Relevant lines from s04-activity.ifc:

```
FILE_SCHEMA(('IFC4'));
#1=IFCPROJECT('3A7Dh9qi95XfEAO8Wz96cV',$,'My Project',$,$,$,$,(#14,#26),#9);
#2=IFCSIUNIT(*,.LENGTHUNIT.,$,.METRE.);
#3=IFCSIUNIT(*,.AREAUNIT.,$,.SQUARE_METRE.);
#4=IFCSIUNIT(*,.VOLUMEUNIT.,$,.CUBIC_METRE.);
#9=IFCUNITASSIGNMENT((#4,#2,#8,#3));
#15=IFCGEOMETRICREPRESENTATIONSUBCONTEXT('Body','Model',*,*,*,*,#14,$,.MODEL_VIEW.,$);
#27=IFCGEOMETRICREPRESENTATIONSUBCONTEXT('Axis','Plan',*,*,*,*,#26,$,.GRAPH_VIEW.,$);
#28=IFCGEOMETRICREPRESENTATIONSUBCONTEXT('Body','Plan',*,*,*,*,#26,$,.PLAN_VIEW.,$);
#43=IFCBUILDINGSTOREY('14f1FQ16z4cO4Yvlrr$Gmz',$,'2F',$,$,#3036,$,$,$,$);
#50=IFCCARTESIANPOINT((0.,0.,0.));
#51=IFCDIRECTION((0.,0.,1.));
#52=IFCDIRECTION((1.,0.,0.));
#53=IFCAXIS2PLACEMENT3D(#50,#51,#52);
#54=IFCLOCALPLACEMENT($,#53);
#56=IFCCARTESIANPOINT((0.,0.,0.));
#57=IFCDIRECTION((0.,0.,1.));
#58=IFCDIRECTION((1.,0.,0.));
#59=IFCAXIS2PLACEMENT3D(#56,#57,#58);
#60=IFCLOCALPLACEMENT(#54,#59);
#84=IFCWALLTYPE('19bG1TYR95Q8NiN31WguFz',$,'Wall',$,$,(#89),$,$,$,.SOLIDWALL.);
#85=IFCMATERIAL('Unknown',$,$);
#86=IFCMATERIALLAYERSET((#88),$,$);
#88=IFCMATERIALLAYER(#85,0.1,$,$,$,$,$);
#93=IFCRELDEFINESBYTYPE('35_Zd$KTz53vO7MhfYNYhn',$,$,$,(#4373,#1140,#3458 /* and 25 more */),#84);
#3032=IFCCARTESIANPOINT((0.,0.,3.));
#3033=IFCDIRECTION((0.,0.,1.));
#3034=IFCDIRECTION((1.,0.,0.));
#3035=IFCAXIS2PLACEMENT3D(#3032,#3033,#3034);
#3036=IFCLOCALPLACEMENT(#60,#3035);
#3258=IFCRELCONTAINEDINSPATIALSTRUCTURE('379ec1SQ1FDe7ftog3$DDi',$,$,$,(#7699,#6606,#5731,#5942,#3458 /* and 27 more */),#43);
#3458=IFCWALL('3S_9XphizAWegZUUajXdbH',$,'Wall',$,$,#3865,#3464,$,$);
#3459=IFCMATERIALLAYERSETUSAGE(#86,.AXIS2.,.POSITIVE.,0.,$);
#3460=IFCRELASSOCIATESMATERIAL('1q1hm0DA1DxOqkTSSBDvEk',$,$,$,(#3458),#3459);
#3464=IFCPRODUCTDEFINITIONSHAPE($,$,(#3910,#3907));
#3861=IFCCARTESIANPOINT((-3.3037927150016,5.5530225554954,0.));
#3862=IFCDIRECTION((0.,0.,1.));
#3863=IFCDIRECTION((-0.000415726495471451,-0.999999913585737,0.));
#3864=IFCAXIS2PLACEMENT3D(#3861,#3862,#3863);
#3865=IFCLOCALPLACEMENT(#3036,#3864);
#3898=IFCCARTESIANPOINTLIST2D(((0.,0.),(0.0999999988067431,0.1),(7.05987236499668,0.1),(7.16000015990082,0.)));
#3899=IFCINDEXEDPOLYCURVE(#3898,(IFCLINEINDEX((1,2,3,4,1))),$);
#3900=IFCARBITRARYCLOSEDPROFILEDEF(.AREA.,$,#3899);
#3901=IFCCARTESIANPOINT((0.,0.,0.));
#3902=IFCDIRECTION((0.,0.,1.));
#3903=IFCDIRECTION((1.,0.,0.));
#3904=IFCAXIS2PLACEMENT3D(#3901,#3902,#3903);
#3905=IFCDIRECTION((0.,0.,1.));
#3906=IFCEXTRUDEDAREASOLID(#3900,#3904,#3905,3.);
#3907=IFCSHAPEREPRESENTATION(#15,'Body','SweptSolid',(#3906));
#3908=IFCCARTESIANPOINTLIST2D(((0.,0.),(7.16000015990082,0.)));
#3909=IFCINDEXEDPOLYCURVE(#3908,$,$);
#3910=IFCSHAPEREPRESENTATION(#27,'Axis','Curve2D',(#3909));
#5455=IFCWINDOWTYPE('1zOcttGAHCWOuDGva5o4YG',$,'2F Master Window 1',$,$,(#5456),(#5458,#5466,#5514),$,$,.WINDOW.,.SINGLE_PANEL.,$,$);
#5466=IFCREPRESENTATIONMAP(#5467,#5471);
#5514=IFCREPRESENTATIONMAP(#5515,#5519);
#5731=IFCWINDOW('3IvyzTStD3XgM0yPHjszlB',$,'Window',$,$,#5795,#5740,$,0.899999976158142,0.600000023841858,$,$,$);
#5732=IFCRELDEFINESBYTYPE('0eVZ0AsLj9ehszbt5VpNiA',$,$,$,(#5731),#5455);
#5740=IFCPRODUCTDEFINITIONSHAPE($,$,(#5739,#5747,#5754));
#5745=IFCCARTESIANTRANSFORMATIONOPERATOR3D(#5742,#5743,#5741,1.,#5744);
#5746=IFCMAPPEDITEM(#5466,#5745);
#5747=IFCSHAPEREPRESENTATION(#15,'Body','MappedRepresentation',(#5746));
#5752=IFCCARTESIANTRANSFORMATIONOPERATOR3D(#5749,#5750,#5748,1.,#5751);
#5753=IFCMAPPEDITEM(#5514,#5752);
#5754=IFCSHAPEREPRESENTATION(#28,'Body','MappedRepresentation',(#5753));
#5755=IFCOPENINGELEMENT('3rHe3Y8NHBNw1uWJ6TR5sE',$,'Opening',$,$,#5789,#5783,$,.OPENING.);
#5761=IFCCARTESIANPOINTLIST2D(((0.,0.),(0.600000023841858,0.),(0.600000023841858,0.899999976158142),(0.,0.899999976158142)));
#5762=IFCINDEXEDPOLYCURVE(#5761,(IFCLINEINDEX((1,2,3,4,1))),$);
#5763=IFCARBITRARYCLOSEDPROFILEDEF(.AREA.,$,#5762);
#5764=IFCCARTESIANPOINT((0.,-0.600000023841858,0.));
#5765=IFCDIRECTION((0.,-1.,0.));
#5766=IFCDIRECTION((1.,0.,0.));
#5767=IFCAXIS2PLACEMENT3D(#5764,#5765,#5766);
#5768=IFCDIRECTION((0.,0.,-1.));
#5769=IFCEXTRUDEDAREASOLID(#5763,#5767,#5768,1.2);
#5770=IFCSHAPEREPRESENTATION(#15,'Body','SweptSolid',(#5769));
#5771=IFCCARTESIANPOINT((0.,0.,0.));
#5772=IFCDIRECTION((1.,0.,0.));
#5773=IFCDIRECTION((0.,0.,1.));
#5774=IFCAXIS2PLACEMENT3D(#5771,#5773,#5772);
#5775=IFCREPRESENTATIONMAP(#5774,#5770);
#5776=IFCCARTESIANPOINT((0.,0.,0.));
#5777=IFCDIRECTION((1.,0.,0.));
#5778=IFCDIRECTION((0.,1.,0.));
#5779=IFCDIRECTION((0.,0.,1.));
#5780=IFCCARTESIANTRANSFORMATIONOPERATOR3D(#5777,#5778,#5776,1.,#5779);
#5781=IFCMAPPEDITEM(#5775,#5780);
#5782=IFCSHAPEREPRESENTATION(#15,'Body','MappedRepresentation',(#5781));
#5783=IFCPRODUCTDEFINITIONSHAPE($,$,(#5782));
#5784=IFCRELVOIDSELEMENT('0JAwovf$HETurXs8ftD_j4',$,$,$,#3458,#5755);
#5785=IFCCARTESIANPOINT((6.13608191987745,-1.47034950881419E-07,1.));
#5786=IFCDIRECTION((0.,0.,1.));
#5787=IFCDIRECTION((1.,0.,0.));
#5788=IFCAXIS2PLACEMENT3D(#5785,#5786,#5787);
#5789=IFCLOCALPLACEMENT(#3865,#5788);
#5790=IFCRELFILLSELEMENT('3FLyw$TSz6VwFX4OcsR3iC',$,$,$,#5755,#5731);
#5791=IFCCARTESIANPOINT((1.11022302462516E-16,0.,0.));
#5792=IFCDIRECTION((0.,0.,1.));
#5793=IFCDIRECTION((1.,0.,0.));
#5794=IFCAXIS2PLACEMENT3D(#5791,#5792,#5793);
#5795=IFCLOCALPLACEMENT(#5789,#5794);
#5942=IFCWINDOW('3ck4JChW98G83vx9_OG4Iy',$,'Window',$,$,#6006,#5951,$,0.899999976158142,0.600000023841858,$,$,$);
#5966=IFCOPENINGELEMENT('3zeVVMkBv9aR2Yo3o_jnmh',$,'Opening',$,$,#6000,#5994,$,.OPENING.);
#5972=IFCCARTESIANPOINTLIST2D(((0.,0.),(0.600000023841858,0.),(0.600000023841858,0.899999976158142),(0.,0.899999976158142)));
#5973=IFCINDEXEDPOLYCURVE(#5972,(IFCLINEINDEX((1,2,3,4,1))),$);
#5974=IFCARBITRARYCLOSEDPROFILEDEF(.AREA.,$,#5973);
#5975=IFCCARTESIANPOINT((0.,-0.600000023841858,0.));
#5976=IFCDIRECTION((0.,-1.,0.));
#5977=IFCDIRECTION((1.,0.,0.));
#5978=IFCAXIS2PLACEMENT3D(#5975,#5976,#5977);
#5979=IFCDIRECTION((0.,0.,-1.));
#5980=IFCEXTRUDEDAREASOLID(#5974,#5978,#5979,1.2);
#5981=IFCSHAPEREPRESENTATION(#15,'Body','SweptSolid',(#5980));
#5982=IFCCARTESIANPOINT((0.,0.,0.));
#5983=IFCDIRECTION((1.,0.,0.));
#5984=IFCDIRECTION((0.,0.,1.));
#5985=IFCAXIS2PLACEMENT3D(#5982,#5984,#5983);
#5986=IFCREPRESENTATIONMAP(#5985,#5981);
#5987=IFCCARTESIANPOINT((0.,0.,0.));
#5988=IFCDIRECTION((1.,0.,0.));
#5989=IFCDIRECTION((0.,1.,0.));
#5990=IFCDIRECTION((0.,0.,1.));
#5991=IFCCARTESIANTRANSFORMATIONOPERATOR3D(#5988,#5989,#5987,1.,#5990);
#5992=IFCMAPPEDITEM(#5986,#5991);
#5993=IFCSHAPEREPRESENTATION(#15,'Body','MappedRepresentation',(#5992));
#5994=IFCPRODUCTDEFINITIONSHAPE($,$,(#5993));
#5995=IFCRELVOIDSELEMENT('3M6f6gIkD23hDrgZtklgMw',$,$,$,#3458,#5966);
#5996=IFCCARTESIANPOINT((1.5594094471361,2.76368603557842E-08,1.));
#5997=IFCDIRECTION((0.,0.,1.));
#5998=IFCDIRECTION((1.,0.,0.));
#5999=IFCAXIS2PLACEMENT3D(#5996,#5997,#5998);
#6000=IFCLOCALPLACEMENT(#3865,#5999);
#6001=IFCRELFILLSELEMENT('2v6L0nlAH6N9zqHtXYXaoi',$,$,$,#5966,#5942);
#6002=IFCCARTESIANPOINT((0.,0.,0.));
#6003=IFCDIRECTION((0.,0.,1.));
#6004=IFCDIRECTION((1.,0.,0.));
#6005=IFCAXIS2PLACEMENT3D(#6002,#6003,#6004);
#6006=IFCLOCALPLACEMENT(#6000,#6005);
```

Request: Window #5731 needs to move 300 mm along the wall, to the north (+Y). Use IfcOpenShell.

```python
import ifcopenshell
import ifcopenshell.api.geometry
import ifcopenshell.util.placement
import ifcopenshell.util.unit

model = ifcopenshell.open("s04-activity.ifc")
unit_scale = ifcopenshell.util.unit.calculate_unit_scale(model)

window = model.by_guid("3IvyzTStD3XgM0yPHjszlB")
opening = window.FillsVoids[0].RelatingOpeningElement
wall = opening.VoidsElements[0].RelatingBuildingElement

wall_matrix = ifcopenshell.util.placement.get_local_placement(wall.ObjectPlacement)
shift = wall_matrix[:3, 0] * -0.3 / unit_scale
before = ifcopenshell.util.placement.get_local_placement(window.ObjectPlacement)[:3, 3].copy()

# The window is placed relative to its opening, so it follows when the opening moves.
matrix = ifcopenshell.util.placement.get_local_placement(opening.ObjectPlacement)
matrix[:3, 3] += shift
ifcopenshell.api.geometry.edit_object_placement(
    model, product=opening, matrix=matrix, is_si=False, should_transform_children=True
)

after = ifcopenshell.util.placement.get_local_placement(window.ObjectPlacement)[:3, 3]
print("window moved by", (after - before).round(3) + 0.0)

model.write("s04-activity_updated.ifc")
```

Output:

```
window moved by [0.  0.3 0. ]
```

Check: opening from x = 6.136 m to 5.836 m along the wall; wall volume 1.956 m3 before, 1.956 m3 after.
